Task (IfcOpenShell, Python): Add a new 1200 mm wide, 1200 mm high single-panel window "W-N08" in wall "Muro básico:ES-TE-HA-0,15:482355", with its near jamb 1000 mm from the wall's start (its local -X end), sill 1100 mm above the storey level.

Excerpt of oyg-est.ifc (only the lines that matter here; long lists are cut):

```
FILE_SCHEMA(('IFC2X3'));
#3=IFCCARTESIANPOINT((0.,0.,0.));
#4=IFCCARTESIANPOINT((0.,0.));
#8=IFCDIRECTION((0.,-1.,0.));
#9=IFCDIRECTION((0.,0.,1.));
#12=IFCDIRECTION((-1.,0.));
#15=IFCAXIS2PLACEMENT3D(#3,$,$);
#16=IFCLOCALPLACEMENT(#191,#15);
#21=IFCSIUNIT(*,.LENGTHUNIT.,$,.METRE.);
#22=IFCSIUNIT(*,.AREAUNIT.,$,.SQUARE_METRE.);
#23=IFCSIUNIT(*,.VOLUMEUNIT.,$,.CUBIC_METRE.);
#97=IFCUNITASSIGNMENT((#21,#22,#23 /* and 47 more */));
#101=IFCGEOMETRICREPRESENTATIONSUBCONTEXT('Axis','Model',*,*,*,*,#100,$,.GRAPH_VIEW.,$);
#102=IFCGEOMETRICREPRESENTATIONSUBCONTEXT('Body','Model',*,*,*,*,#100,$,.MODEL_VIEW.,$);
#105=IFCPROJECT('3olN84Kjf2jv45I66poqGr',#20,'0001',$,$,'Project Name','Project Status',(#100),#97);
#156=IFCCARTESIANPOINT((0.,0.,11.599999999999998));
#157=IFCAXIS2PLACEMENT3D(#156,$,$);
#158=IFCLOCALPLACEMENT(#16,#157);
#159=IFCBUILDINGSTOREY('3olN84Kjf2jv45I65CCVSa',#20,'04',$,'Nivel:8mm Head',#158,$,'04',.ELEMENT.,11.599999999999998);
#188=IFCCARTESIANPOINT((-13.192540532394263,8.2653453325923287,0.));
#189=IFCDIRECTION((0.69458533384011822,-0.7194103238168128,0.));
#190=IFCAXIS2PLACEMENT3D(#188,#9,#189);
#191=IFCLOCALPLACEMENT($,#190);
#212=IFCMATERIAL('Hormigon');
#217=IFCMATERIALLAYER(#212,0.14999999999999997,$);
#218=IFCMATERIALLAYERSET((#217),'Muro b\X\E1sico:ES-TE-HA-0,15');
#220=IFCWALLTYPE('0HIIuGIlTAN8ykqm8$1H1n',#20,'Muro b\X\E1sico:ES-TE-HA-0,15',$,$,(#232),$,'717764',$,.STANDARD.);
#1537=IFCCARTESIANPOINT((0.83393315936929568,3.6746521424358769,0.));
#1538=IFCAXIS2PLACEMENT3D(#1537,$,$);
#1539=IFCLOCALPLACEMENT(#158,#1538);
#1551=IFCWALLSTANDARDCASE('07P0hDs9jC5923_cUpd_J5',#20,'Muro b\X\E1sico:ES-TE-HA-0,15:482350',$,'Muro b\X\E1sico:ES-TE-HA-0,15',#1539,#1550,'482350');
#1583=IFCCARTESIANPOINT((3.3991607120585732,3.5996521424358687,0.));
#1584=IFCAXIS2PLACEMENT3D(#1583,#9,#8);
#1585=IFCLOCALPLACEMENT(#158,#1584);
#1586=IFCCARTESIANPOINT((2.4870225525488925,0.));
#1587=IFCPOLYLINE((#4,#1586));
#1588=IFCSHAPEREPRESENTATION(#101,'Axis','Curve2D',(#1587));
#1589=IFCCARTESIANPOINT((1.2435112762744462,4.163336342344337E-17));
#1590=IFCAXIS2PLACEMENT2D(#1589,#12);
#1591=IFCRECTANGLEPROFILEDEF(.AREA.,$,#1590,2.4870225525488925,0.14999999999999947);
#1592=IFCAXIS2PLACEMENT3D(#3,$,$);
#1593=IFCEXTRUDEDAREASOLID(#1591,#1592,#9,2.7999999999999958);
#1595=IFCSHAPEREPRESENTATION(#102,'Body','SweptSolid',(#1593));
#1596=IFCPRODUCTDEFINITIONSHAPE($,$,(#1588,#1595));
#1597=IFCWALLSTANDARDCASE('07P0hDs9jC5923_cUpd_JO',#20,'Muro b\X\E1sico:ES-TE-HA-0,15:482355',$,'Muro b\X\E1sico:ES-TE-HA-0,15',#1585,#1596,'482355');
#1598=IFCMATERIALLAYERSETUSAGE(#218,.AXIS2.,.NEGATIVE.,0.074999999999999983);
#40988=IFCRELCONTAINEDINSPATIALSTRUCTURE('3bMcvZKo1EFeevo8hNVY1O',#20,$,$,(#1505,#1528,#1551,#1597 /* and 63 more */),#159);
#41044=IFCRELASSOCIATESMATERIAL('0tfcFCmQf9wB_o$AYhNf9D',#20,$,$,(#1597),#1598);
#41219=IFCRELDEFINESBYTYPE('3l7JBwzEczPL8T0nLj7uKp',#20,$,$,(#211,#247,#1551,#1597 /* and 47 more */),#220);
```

```python
import numpy as np
import ifcopenshell
import ifcopenshell.api.feature
import ifcopenshell.api.geometry
import ifcopenshell.api.root
import ifcopenshell.api.spatial
import ifcopenshell.api.type
import ifcopenshell.geom
import ifcopenshell.util.element
import ifcopenshell.util.placement
import ifcopenshell.util.representation
import ifcopenshell.util.shape
import ifcopenshell.util.unit

model = ifcopenshell.open("oyg-est.ifc")
unit_scale = ifcopenshell.util.unit.calculate_unit_scale(model)
settings = ifcopenshell.geom.settings()


def volume(element):
    """Net volume in cubic metres, openings subtracted."""
    shape = ifcopenshell.geom.create_shape(settings, element)
    return ifcopenshell.util.shape.get_volume(shape.geometry)


wall = model.by_id(1597)
storey = ifcopenshell.util.element.get_container(wall, ifc_class="IfcBuildingStorey")
context = ifcopenshell.util.representation.get_context(model, "Model", "Body", "MODEL_VIEW")
before = volume(wall)

width, height, from_end, sill = 1.2, 1.2, 1, 1.1  # metres

# The wall runs along its own X axis, and the end named is its -X end.
wall_shape = ifcopenshell.geom.create_shape(settings, wall)
x, y, z = ifcopenshell.util.shape.get_vertices(wall_shape.geometry).T
start = x.min() + from_end
face, thickness = float(y.min()), float(y.max() - y.min())
wall_matrix = ifcopenshell.util.placement.get_local_placement(wall.ObjectPlacement)
level = ifcopenshell.util.placement.get_local_placement(storey.ObjectPlacement)[2, 3]


def in_wall(x, y):
    """Placement at x, y metres in the wall's axes, at sill height."""
    matrix = wall_matrix.copy()
    matrix[:, 3] = wall_matrix @ np.array([x / unit_scale, y / unit_scale, 0.0, 1.0])
    matrix[2, 3] = level + sill / unit_scale
    return matrix


# Opening: a box that overshoots both wall faces by 50 mm.
opening = ifcopenshell.api.root.create_entity(model, ifc_class="IfcOpeningElement")
box = ifcopenshell.api.geometry.add_wall_representation(
    model, context=context, length=width, height=height, thickness=thickness + 0.1
)
ifcopenshell.api.geometry.assign_representation(model, product=opening, representation=box)
ifcopenshell.api.geometry.edit_object_placement(model, product=opening, matrix=in_wall(start, face - 0.05), is_si=False)
ifcopenshell.api.feature.add_feature(model, feature=opening, element=wall)

window = ifcopenshell.api.root.create_entity(model, ifc_class="IfcWindow", name="W-N08")
window.OverallWidth, window.OverallHeight = width / unit_scale, height / unit_scale
body = ifcopenshell.api.geometry.add_window_representation(
    model,
    context=context,
    overall_width=window.OverallWidth,
    overall_height=window.OverallHeight,
    partition_type="SINGLE_PANEL",
)
ifcopenshell.api.geometry.assign_representation(model, product=window, representation=body)
ifcopenshell.api.spatial.assign_container(model, products=[window], relating_structure=storey)
fills = ifcopenshell.api.feature.add_filling(model, opening=opening, element=window)
fills.OwnerHistory = window.OwnerHistory  # required in IFC2X3

# IFC2X3 keeps the operation on the window style.
style = ifcopenshell.api.root.create_entity(model, ifc_class="IfcWindowStyle", name="W-N08")
style.OperationType, style.ConstructionType = "SINGLE_PANEL", "NOTDEFINED"
style.ParameterTakesPrecedence = style.Sizeable = False
ifcopenshell.api.type.assign_type(model, related_objects=[window], relating_type=style)

# Centre the window in the wall's thickness.
ifcopenshell.api.geometry.edit_object_placement(model, product=window, matrix=in_wall(start, face), is_si=False)
window_shape = ifcopenshell.geom.create_shape(settings, window)
depth = ifcopenshell.util.shape.get_vertices(window_shape.geometry)[:, 1]
offset = face + thickness / 2 - (depth.min() + depth.max()) / 2
ifcopenshell.api.geometry.edit_object_placement(model, product=window, matrix=in_wall(start, offset), is_si=False)

after = volume(wall)

print(f"wall volume {before:.3f} -> {after:.3f} m3")

model.write("oyg-est_rev.ifc")
```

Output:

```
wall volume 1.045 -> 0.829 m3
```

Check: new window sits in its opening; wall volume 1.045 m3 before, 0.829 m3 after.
